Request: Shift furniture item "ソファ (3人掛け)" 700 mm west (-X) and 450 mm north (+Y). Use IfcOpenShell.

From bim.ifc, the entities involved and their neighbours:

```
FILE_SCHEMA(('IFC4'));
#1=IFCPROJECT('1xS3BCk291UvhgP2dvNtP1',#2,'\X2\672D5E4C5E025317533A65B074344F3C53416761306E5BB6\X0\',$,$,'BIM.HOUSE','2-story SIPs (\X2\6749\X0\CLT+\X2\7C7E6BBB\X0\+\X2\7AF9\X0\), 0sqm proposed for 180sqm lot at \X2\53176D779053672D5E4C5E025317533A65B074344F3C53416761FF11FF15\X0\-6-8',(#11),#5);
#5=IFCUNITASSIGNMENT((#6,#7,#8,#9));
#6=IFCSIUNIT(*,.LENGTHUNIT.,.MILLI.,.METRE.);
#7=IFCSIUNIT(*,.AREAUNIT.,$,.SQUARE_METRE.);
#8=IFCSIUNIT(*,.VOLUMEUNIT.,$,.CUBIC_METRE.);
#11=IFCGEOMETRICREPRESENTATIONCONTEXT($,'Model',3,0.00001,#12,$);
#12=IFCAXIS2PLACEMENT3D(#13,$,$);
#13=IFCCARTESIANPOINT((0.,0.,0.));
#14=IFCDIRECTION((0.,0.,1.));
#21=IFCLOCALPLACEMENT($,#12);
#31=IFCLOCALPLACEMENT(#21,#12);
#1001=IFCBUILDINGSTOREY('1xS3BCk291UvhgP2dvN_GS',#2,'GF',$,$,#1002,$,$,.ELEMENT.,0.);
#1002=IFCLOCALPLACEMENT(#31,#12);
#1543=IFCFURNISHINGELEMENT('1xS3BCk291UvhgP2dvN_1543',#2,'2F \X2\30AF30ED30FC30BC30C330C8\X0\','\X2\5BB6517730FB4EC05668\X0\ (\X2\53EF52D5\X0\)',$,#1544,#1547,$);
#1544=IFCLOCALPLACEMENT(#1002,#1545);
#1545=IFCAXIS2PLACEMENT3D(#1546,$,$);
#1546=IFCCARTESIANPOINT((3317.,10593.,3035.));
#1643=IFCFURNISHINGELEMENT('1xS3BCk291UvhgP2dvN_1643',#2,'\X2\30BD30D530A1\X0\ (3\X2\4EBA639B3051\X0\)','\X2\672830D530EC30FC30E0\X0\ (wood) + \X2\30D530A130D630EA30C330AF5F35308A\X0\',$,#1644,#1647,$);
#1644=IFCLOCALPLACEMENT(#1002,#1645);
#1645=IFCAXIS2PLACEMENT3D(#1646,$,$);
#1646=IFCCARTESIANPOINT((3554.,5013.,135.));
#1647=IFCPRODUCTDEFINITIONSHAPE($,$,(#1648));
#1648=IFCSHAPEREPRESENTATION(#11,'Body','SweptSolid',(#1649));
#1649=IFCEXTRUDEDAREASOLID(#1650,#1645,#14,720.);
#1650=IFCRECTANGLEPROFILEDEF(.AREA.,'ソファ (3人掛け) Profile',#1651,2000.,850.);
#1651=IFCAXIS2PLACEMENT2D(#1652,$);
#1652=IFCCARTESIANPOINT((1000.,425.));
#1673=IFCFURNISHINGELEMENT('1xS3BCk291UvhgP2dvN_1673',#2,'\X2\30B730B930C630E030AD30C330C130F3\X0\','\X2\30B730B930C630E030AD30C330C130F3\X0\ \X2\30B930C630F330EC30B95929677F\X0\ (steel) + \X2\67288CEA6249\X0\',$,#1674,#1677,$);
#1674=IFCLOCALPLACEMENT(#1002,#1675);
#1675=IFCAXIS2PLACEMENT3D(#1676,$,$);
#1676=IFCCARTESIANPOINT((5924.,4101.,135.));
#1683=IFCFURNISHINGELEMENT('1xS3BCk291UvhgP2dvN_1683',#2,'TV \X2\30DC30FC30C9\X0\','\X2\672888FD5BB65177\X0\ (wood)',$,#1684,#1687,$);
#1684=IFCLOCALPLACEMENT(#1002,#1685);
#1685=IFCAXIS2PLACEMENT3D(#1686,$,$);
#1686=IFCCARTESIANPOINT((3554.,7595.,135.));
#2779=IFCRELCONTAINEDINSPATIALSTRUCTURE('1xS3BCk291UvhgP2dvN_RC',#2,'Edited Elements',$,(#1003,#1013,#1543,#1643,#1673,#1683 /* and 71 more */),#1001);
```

```python
import ifcopenshell
import ifcopenshell.api.geometry
import ifcopenshell.util.placement
import ifcopenshell.util.unit

model = ifcopenshell.open("bim.ifc")
unit_scale = ifcopenshell.util.unit.calculate_unit_scale(model)

item = model.by_guid("1xS3BCk291UvhgP2dvN_1643")
matrix = ifcopenshell.util.placement.get_local_placement(item.ObjectPlacement)
matrix[0, 3] -= 0.7 / unit_scale
matrix[1, 3] += 0.45 / unit_scale
ifcopenshell.api.geometry.edit_object_placement(model, product=item, matrix=matrix, is_si=False)

print(ifcopenshell.util.placement.get_local_placement(item.ObjectPlacement).round(3) + 0.0)

model.write("bim_rev.ifc")
```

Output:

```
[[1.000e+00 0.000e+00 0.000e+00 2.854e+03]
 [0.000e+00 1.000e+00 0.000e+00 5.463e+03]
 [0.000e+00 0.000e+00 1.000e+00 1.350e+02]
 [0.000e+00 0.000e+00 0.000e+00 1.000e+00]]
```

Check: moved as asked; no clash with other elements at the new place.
